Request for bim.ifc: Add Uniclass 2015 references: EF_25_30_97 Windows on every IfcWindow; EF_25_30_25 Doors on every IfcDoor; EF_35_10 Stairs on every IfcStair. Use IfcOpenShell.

First a look at what the model holds.

```python
import ifcopenshell

model = ifcopenshell.open("bim.ifc")
print(model.schema)
print("classifications:", [c.Name for c in model.by_type("IfcClassification")])
for ifc_class in ("IfcDoor", "IfcRoof", "IfcStair", "IfcWall", "IfcWindow"):
    print(ifc_class, len(model.by_type(ifc_class)))
```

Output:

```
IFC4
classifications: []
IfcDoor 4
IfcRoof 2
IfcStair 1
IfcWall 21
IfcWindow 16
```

```python
import ifcopenshell
import ifcopenshell.api.classification

model = ifcopenshell.open("bim.ifc")

system = ifcopenshell.api.classification.add_classification(model, classification="Uniclass 2015")

codes = {
    "IfcWindow": ("EF_25_30_97", "Windows"),
    "IfcDoor": ("EF_25_30_25", "Doors"),
    "IfcStair": ("EF_35_10", "Stairs"),
}
for ifc_class, (code, name) in codes.items():
    products = model.by_type(ifc_class)
    ifcopenshell.api.classification.add_reference(
        model, products=products, classification=system, identification=code, name=name
    )
    print(code, len(products))

model.write("bim_edited.ifc")
```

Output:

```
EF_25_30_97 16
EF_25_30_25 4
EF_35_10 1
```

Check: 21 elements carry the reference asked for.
